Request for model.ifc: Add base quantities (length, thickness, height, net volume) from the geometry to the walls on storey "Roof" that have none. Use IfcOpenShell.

First a look at what the model holds.

```python
import ifcopenshell
import ifcopenshell.util.element
import ifcopenshell.util.unit

model = ifcopenshell.open("model.ifc")
print(model.schema)
for unit_type in ("LENGTHUNIT", "AREAUNIT", "VOLUMEUNIT"):
    print(unit_type, ifcopenshell.util.unit.calculate_unit_scale(model, unit_type))
storey = next(s for s in model.by_type("IfcBuildingStorey") if s.Name == "Roof")
walls = [e for e in ifcopenshell.util.element.get_decomposition(storey) if e.is_a("IfcWall")]
for e in sorted(walls, key=lambda e: e.id()):
    print(e.id(), e.is_a(), e.Name, list(ifcopenshell.util.element.get_psets(e, qtos_only=True)), sep=" | ")
```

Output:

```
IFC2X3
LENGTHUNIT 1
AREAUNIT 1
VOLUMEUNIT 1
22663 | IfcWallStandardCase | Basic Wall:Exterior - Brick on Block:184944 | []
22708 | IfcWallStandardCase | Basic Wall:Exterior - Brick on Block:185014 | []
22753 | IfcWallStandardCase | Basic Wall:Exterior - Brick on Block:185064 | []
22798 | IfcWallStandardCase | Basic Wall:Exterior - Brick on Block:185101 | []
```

```python
import ifcopenshell
import ifcopenshell.api.pset
import ifcopenshell.geom
import ifcopenshell.util.element
import ifcopenshell.util.shape
import ifcopenshell.util.unit

model = ifcopenshell.open("model.ifc")
unit_scale = ifcopenshell.util.unit.calculate_unit_scale(model)
volume_scale = ifcopenshell.util.unit.calculate_unit_scale(model, "VOLUMEUNIT")
settings = ifcopenshell.geom.settings()

storey = next(s for s in model.by_type("IfcBuildingStorey") if s.Name == "Roof")
walls = [e for e in ifcopenshell.util.element.get_decomposition(storey) if e.is_a("IfcWall")]

for e in sorted(walls, key=lambda e: e.id()):
    if ifcopenshell.util.element.get_psets(e, qtos_only=True, should_inherit=False):
        continue
    # Geometry comes back in metres, in the element's own axes.
    shape = ifcopenshell.geom.create_shape(settings, e)
    values = {
        "Length": ifcopenshell.util.shape.get_x(shape.geometry) / unit_scale,
        "Width": ifcopenshell.util.shape.get_y(shape.geometry) / unit_scale,
        "Height": ifcopenshell.util.shape.get_z(shape.geometry) / unit_scale,
        "NetVolume": ifcopenshell.util.shape.get_volume(shape.geometry) / volume_scale,
    }
    qto = ifcopenshell.api.pset.add_qto(model, product=e, name="BaseQuantities")
    ifcopenshell.api.pset.edit_qto(model, qto=qto, properties=values)
    print(e.id(), {k: round(v, 3) for k, v in values.items()})

model.write("model-out.ifc")
```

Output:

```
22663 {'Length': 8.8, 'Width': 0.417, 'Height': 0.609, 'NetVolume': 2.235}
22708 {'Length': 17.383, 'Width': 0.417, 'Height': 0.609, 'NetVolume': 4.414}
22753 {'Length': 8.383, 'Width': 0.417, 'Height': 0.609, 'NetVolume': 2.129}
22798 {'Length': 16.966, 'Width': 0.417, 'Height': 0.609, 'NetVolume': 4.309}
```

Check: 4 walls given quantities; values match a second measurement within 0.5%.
